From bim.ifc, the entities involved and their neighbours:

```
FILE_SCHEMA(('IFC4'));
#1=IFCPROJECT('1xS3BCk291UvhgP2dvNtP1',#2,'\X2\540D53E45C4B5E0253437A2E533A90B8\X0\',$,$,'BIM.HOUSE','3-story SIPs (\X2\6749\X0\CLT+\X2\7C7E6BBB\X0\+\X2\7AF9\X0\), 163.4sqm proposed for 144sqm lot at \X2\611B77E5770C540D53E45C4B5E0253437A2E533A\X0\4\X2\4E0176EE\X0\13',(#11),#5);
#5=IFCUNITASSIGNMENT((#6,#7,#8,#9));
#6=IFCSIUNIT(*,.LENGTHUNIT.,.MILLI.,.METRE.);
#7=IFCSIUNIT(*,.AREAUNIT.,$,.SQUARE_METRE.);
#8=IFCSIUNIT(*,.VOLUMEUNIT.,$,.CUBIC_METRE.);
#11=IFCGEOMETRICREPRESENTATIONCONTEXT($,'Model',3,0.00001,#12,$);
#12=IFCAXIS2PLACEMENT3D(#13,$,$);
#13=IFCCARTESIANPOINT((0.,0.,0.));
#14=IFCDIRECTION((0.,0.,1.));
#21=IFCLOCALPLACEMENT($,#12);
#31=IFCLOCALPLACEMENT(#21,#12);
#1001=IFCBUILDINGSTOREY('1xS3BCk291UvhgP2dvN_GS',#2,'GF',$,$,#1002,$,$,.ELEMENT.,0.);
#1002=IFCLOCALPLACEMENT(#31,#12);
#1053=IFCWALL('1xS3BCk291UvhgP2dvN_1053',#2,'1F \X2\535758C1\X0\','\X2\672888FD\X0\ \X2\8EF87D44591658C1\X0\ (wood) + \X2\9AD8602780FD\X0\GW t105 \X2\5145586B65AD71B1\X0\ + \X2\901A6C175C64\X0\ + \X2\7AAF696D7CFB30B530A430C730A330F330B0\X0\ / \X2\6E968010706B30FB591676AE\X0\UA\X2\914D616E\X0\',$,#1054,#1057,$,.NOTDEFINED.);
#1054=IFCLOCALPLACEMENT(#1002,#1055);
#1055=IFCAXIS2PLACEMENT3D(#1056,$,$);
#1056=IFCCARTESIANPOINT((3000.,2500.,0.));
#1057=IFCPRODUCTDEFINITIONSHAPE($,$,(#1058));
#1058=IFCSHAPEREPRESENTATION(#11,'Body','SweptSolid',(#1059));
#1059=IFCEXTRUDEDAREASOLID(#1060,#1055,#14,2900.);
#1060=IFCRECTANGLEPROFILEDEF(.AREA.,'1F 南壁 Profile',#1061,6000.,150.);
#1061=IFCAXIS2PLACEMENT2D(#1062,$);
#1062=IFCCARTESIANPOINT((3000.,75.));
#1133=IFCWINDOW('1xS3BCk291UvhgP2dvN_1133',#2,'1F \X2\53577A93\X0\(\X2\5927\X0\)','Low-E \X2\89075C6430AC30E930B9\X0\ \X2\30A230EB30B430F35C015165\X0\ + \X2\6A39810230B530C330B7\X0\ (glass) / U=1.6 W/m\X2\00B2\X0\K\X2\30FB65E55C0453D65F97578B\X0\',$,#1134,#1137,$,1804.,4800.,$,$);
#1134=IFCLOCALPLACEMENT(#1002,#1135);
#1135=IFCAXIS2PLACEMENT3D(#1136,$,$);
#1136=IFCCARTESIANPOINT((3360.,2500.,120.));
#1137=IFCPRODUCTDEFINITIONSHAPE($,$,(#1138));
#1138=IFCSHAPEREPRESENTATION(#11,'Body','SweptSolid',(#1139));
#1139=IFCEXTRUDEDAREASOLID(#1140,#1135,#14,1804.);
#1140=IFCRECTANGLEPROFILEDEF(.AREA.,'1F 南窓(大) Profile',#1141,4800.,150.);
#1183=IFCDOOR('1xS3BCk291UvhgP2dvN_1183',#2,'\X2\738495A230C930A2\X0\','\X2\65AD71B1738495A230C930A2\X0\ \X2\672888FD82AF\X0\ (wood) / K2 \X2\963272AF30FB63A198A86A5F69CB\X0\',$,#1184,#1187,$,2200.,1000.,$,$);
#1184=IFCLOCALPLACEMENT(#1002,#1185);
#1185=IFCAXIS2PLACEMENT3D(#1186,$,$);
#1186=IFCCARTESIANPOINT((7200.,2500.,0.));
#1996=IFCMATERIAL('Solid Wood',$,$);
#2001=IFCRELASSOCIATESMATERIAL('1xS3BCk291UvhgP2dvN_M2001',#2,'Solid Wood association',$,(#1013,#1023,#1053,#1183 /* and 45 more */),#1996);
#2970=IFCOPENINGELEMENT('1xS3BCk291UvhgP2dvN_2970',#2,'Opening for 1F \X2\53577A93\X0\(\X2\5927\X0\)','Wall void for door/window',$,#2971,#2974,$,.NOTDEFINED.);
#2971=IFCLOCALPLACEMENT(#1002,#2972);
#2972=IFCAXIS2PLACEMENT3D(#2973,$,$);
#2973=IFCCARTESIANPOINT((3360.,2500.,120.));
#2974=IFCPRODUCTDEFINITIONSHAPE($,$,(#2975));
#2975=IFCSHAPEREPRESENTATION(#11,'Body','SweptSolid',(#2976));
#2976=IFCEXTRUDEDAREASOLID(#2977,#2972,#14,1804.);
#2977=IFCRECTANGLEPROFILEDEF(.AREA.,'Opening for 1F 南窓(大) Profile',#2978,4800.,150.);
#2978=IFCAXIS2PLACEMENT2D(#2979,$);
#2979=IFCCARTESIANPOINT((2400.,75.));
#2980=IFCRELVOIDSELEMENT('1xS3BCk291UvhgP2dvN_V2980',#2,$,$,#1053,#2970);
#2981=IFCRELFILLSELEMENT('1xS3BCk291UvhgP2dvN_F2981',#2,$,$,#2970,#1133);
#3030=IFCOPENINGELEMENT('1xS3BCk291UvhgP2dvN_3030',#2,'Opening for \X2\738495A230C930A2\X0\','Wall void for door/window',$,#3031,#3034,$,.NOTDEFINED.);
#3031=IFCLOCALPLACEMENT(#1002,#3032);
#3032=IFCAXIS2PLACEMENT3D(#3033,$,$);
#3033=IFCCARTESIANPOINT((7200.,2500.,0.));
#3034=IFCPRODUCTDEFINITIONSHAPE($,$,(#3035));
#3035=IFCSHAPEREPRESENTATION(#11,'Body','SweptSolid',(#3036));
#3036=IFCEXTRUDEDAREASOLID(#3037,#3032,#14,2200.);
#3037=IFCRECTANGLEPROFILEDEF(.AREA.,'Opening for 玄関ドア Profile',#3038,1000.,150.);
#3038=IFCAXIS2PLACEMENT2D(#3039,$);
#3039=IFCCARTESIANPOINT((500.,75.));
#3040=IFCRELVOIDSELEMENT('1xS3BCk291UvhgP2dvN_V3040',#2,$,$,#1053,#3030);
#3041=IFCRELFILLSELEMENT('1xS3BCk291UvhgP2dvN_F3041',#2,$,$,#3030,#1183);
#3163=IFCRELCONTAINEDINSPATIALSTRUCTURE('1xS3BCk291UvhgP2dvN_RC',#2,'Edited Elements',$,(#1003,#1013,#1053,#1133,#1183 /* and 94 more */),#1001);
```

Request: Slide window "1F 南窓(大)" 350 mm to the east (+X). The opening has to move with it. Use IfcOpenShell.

```python
import ifcopenshell
import ifcopenshell.api.geometry
import ifcopenshell.util.placement
import ifcopenshell.util.unit

model = ifcopenshell.open("bim.ifc")
unit_scale = ifcopenshell.util.unit.calculate_unit_scale(model)

window = model.by_guid("1xS3BCk291UvhgP2dvN_1133")
opening = window.FillsVoids[0].RelatingOpeningElement
wall = opening.VoidsElements[0].RelatingBuildingElement

wall_matrix = ifcopenshell.util.placement.get_local_placement(wall.ObjectPlacement)
shift = wall_matrix[:3, 0] * 0.35 / unit_scale
before = ifcopenshell.util.placement.get_local_placement(window.ObjectPlacement)[:3, 3].copy()

# The window is not placed relative to its opening, so move both.
for product in (opening, window):
    matrix = ifcopenshell.util.placement.get_local_placement(product.ObjectPlacement)
    matrix[:3, 3] += shift
    ifcopenshell.api.geometry.edit_object_placement(model, product=product, matrix=matrix, is_si=False)

after = ifcopenshell.util.placement.get_local_placement(window.ObjectPlacement)[:3, 3]
print("window moved by", (after - before).round(3) + 0.0)

model.write("bim_rev.ifc")
```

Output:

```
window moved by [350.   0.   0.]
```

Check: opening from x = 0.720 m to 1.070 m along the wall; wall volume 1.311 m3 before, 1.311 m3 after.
